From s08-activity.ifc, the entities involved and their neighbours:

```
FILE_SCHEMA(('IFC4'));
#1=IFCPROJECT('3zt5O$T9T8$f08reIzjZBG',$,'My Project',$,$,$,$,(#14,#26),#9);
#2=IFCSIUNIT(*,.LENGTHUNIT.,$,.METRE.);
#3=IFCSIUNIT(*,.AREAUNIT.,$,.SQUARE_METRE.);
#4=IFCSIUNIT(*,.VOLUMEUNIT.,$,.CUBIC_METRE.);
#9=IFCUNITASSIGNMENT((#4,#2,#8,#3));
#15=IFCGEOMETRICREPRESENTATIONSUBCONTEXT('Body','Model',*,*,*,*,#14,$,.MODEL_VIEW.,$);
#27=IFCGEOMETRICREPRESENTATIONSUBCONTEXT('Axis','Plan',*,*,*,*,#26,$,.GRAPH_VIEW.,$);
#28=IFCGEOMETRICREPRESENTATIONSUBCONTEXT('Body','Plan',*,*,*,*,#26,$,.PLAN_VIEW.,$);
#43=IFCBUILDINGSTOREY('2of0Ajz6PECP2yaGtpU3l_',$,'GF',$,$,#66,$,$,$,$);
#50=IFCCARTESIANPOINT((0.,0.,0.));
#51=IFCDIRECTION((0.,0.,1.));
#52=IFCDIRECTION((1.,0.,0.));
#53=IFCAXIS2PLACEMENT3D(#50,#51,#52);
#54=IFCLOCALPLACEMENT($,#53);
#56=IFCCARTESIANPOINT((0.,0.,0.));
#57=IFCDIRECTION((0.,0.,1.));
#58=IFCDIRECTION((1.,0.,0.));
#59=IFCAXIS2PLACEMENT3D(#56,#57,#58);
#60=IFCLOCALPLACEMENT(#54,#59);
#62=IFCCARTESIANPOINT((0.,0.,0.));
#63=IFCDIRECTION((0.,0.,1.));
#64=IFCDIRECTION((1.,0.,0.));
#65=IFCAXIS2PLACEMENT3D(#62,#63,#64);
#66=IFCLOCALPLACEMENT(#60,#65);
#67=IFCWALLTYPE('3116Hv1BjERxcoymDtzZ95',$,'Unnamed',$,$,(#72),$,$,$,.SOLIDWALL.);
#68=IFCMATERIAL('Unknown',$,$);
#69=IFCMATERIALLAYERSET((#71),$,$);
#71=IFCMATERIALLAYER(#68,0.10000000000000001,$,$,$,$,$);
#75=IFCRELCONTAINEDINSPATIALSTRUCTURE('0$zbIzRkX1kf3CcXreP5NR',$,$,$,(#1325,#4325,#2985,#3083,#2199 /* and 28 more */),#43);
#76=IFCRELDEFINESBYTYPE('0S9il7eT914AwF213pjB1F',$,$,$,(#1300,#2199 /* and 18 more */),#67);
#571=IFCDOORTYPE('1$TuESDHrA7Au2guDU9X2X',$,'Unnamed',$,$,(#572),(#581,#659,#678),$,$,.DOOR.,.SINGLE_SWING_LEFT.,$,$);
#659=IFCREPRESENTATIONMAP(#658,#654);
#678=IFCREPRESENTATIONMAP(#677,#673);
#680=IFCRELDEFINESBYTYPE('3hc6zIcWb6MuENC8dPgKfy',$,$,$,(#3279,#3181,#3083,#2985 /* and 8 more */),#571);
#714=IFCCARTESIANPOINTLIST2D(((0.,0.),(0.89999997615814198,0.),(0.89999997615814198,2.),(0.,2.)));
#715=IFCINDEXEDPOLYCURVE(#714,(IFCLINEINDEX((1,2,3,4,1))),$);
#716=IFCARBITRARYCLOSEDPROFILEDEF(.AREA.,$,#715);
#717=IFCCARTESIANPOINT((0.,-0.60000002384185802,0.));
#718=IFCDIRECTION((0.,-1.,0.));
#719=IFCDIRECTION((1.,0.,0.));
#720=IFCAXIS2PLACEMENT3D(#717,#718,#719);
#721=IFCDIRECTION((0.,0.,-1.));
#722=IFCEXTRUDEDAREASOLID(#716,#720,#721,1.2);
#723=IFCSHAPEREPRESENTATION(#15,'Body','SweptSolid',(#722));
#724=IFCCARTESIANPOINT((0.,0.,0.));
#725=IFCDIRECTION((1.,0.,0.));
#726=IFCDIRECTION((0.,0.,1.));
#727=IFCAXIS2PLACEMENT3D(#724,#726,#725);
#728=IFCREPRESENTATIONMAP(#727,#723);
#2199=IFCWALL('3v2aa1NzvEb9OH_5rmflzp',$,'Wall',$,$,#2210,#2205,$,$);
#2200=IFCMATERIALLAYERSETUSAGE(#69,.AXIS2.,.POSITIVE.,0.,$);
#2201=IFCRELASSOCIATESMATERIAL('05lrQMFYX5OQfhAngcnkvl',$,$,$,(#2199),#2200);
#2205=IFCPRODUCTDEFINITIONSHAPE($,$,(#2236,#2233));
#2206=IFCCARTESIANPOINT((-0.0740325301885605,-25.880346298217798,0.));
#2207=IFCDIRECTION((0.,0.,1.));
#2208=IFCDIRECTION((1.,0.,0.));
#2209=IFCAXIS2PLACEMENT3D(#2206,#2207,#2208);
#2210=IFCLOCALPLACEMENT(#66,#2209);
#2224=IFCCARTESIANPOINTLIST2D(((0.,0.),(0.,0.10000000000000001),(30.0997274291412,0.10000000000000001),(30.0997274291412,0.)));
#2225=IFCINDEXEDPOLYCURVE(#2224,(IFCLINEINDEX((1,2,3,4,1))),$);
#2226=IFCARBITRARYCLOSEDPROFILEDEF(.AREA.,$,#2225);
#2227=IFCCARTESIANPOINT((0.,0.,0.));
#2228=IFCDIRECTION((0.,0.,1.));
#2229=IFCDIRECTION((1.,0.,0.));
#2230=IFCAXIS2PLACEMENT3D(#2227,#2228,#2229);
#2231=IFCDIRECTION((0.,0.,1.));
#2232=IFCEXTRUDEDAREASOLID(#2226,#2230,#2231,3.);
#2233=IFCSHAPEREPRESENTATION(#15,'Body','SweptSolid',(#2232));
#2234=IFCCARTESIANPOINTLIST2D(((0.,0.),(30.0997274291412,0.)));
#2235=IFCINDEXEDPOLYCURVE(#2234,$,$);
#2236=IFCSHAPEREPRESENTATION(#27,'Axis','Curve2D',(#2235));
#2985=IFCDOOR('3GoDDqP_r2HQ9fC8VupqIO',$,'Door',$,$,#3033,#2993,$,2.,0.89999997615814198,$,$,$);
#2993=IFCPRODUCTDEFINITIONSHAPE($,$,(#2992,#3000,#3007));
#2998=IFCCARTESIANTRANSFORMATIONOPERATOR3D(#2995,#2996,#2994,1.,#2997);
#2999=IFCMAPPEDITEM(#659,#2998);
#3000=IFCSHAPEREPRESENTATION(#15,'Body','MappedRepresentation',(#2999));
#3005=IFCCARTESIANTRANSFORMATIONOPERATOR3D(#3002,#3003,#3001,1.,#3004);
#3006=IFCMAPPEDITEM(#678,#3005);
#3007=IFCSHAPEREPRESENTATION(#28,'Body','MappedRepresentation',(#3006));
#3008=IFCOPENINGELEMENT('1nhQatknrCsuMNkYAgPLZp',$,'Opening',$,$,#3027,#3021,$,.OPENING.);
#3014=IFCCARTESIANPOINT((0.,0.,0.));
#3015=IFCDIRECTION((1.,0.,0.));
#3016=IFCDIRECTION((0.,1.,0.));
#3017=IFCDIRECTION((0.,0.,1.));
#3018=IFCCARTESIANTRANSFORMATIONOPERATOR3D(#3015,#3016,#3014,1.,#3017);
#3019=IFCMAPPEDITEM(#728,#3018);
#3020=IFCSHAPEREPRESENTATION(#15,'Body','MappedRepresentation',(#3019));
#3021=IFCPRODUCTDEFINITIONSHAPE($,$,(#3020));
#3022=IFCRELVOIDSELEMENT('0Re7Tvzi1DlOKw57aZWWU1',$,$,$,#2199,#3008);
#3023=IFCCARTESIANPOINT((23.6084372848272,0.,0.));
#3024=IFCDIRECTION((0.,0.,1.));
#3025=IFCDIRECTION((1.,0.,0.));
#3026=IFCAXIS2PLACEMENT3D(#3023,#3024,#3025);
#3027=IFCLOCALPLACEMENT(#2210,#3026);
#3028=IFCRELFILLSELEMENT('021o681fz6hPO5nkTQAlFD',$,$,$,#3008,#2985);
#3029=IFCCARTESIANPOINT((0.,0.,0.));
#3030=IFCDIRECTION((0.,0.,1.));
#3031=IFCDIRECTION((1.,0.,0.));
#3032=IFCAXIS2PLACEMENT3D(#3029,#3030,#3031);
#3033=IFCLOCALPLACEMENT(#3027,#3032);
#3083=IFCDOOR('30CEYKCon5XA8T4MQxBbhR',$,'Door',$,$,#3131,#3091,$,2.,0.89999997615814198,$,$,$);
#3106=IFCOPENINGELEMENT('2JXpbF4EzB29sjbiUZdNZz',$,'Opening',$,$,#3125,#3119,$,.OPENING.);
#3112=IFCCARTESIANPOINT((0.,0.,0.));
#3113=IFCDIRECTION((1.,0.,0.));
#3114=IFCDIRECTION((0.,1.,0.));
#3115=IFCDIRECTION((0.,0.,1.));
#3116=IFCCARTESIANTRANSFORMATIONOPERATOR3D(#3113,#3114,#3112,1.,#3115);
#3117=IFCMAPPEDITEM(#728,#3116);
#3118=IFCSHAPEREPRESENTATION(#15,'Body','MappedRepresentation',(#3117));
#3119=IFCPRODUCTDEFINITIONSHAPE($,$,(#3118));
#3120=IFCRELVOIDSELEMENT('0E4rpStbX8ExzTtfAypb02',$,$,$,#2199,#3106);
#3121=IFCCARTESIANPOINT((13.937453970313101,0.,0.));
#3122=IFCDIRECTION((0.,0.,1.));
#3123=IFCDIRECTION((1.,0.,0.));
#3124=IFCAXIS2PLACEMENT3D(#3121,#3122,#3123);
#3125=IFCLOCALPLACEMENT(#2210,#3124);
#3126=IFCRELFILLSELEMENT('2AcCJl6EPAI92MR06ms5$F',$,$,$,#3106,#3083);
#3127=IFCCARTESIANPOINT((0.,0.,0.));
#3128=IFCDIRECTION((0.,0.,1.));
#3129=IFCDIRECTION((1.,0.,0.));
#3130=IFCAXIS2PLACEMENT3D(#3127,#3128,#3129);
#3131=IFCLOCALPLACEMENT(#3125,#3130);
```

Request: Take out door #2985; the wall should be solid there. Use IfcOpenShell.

```python
import ifcopenshell
import ifcopenshell.api.feature
import ifcopenshell.api.root
import ifcopenshell.geom
import ifcopenshell.util.shape

model = ifcopenshell.open("s08-activity.ifc")
settings = ifcopenshell.geom.settings()


def volume(element):
    """Net volume in cubic metres, openings subtracted."""
    shape = ifcopenshell.geom.create_shape(settings, element)
    return ifcopenshell.util.shape.get_volume(shape.geometry)


door = model.by_id(2985)
opening = door.FillsVoids[0].RelatingOpeningElement
wall = opening.VoidsElements[0].RelatingBuildingElement
before = volume(wall)

ifcopenshell.api.root.remove_product(model, product=door)
ifcopenshell.api.feature.remove_feature(model, feature=opening)

after = volume(wall)

print(f"wall volume {before:.3f} -> {after:.3f} m3")

model.write("s08-activity_updated.ifc")
```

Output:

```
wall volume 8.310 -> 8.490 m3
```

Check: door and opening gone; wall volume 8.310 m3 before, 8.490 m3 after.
